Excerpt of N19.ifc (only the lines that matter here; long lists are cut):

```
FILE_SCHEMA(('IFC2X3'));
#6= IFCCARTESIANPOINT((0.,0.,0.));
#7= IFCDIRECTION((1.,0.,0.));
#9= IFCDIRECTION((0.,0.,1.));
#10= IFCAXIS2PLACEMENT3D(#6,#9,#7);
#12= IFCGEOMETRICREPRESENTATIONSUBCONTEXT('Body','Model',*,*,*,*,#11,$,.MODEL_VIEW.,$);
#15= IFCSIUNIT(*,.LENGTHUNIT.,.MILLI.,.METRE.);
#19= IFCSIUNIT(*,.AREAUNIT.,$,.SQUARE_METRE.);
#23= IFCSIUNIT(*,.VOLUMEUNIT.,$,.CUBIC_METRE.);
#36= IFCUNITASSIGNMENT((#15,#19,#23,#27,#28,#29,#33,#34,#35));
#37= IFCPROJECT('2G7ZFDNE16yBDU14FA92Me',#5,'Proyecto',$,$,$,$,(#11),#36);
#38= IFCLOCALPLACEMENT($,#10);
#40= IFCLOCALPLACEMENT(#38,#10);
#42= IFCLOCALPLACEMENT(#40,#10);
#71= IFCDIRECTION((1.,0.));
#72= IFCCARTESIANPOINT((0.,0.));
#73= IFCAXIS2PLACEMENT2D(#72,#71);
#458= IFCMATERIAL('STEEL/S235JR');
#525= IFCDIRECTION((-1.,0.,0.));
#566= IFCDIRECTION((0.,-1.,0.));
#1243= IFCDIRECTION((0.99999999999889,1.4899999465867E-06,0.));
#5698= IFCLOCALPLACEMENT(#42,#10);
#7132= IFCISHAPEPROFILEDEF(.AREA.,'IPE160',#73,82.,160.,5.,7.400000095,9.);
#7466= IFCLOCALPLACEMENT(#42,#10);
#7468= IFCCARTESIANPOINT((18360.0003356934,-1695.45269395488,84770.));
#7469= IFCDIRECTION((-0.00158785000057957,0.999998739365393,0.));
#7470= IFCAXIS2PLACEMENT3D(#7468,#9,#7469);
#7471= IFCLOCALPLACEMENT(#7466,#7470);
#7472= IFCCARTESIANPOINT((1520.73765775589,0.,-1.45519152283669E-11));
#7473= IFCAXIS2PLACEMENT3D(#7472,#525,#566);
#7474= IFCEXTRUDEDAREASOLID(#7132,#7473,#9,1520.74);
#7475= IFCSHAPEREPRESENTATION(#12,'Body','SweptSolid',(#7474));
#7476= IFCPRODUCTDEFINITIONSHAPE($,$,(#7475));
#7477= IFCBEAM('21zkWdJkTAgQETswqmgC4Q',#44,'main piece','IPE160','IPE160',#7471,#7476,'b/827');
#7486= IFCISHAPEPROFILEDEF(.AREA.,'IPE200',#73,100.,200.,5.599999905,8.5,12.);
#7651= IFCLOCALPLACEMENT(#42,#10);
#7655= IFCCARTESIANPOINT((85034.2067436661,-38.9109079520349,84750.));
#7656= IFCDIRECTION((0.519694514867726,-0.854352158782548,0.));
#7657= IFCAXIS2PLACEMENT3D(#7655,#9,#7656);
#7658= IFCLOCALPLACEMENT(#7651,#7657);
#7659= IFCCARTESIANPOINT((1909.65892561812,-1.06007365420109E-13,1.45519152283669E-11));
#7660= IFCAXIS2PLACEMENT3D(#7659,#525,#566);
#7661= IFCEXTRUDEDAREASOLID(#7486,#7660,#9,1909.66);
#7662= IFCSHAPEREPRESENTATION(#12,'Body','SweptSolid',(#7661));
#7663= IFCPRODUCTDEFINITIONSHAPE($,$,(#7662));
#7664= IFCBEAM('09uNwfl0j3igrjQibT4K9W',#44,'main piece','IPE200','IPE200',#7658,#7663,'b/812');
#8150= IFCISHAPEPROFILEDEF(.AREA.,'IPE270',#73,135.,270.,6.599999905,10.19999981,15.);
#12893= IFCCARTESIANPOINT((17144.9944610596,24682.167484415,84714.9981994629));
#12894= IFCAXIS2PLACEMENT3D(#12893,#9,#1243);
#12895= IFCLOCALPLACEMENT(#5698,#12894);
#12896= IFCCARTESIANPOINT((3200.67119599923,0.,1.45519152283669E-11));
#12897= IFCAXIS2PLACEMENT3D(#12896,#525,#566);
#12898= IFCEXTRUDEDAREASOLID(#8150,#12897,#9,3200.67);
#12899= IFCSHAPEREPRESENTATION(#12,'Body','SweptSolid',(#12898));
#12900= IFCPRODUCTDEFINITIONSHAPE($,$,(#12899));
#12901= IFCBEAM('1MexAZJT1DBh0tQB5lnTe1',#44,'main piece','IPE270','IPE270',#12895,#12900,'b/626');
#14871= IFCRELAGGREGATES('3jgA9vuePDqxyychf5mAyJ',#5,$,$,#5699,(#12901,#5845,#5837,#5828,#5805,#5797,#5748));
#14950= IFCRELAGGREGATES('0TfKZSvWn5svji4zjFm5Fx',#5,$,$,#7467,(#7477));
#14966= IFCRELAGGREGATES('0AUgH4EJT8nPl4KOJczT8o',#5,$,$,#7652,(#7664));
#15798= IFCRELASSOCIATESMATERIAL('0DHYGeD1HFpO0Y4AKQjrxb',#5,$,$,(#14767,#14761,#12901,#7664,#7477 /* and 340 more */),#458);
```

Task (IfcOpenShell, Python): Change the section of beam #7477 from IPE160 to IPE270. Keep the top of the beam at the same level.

```python
import ifcopenshell
import ifcopenshell.util.element
import ifcopenshell.util.representation

model = ifcopenshell.open("N19.ifc")

member = model.by_guid("21zkWdJkTAgQETswqmgC4Q")
source = next(p for p in model.by_type("IfcIShapeProfileDef") if p.ProfileName == "IPE270")

body = ifcopenshell.util.representation.get_representation(member, "Model", "Body")
solid = body.Items[0]
old_profile = solid.SweptArea

# Copy the section's sizes but keep this member's own profile position.
profile = ifcopenshell.util.element.copy(model, source)
# Profiles are centred, so shift by half the change in depth to hold the top.
shift = (old_profile.OverallDepth - profile.OverallDepth) / 2
x, y = old_profile.Position.Location.Coordinates
up = (0.0, 1.0)  # upwards, in the solid's own plane
location = model.createIfcCartesianPoint((x + up[0] * shift, y + up[1] * shift))
profile.Position = model.createIfcAxis2Placement2D(location, old_profile.Position.RefDirection)
solid.SweptArea = profile
if not model.get_total_inverses(old_profile):
    ifcopenshell.util.element.remove_deep2(model, old_profile)
member.Description = member.Description.replace("IPE160", "IPE270")
member.ObjectType = member.ObjectType.replace("IPE160", "IPE270")

print(solid.SweptArea)

model.write("N19-out.ifc")
```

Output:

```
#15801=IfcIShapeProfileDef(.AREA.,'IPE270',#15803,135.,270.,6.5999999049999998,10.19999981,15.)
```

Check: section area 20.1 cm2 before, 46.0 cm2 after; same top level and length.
